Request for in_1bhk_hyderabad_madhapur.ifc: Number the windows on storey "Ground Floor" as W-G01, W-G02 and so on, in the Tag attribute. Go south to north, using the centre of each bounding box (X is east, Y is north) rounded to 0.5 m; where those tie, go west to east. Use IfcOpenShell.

First a look at what the model holds.

```python
import ifcopenshell
import ifcopenshell.util.element
import ifcopenshell.util.placement

model = ifcopenshell.open("in_1bhk_hyderabad_madhapur.ifc")
print(model.schema)
storey = next(s for s in model.by_type("IfcBuildingStorey") if s.Name == "Ground Floor")
windows = [e for e in ifcopenshell.util.element.get_decomposition(storey) if e.is_a("IfcWindow")]
for e in sorted(windows, key=lambda e: e.id()):
    origin = ifcopenshell.util.placement.get_local_placement(e.ObjectPlacement)[:3, 3]
    print(e.id(), e.Tag, e.Name, origin.round(2) + 0.0, sep=" | ")
```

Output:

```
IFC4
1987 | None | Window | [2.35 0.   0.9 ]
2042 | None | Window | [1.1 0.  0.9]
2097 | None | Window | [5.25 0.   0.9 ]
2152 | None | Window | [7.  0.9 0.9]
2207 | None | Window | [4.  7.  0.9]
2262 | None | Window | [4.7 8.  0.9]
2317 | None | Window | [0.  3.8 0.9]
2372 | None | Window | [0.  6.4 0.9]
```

```python
import ifcopenshell
import ifcopenshell.geom
import ifcopenshell.util.element
import ifcopenshell.util.shape

model = ifcopenshell.open("in_1bhk_hyderabad_madhapur.ifc")
settings = ifcopenshell.geom.settings()
settings.set("use-world-coords", True)


def centre(element):
    shape = ifcopenshell.geom.create_shape(settings, element)
    return ifcopenshell.util.shape.get_bbox_centroid(shape.geometry)


storey = next(s for s in model.by_type("IfcBuildingStorey") if s.Name == "Ground Floor")
windows = [e for e in ifcopenshell.util.element.get_decomposition(storey) if e.is_a("IfcWindow")]

# Insertion points can sit at a corner or the storey origin, so sort by the geometry (in metres).
centres = {e: centre(e) for e in windows}
windows.sort(key=lambda e: (round(centres[e][1] / 0.5), centres[e][0]))

for i, e in enumerate(windows, start=1):
    number = f"W-G{i:02d}"
    e.Tag = number
    print(e.id(), number)

model.write("in_1bhk_hyderabad_madhapur_updated.ifc")
```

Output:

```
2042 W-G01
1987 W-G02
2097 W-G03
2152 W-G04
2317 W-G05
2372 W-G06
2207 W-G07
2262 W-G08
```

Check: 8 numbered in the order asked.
